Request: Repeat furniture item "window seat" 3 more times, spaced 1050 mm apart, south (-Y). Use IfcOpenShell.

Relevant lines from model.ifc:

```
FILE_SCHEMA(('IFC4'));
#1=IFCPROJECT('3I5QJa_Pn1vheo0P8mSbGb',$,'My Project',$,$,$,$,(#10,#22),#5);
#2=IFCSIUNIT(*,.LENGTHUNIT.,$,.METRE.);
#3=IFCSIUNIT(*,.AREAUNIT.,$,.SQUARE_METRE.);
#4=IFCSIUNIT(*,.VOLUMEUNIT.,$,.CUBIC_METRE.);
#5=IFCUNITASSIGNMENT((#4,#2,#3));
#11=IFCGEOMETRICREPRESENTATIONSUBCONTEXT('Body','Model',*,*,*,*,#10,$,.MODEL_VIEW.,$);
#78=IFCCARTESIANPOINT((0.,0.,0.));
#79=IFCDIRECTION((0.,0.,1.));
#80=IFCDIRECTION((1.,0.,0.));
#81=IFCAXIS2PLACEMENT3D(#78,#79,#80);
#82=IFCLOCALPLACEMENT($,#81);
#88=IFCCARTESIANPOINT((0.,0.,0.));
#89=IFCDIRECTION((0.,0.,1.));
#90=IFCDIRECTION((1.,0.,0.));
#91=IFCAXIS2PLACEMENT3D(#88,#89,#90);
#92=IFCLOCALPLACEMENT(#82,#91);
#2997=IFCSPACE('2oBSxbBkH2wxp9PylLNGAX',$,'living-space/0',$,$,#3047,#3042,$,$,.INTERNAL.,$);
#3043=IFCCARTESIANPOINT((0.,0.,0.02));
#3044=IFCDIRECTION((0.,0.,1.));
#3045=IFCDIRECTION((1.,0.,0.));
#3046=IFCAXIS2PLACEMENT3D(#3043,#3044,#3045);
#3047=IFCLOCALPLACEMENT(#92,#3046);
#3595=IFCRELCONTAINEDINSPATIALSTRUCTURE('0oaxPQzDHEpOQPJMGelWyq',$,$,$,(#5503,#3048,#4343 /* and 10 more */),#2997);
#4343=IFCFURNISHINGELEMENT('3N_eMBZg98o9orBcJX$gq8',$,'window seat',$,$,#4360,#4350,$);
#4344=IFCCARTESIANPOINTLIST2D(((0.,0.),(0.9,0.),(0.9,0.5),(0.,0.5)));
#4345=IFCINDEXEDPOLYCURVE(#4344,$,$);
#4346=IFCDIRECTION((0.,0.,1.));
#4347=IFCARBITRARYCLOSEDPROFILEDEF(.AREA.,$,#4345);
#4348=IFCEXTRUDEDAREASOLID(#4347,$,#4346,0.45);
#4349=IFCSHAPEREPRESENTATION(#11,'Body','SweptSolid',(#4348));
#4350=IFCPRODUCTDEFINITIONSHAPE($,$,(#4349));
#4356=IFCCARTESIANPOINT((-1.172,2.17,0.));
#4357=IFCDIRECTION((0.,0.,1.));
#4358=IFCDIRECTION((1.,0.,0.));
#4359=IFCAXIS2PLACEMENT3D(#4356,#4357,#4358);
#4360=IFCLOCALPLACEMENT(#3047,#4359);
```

```python
import numpy as np
import ifcopenshell
import ifcopenshell.api.geometry
import ifcopenshell.api.root
import ifcopenshell.util.element
import ifcopenshell.util.placement

model = ifcopenshell.open("model.ifc")

source = model.by_id(4343)
base = ifcopenshell.util.placement.get_local_placement(source.ObjectPlacement)
step = np.array([0.0, -1.0, 0.0]) * 1.05

for i in range(1, 4):
    copy = ifcopenshell.api.root.copy_class(model, product=source)
    copy.Representation = ifcopenshell.util.element.copy_deep(
        model, source.Representation, exclude=["IfcGeometricRepresentationContext", "IfcRepresentationMap"]
    )
    matrix = base.copy()
    matrix[:3, 3] += i * step
    print("added at", matrix[:3, 3].round(3) + 0.0)
    ifcopenshell.api.geometry.edit_object_placement(model, product=copy, matrix=matrix, is_si=False)

model.write("model_updated.ifc")
```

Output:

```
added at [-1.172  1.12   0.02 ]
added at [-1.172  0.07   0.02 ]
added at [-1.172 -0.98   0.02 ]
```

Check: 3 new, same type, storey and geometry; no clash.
